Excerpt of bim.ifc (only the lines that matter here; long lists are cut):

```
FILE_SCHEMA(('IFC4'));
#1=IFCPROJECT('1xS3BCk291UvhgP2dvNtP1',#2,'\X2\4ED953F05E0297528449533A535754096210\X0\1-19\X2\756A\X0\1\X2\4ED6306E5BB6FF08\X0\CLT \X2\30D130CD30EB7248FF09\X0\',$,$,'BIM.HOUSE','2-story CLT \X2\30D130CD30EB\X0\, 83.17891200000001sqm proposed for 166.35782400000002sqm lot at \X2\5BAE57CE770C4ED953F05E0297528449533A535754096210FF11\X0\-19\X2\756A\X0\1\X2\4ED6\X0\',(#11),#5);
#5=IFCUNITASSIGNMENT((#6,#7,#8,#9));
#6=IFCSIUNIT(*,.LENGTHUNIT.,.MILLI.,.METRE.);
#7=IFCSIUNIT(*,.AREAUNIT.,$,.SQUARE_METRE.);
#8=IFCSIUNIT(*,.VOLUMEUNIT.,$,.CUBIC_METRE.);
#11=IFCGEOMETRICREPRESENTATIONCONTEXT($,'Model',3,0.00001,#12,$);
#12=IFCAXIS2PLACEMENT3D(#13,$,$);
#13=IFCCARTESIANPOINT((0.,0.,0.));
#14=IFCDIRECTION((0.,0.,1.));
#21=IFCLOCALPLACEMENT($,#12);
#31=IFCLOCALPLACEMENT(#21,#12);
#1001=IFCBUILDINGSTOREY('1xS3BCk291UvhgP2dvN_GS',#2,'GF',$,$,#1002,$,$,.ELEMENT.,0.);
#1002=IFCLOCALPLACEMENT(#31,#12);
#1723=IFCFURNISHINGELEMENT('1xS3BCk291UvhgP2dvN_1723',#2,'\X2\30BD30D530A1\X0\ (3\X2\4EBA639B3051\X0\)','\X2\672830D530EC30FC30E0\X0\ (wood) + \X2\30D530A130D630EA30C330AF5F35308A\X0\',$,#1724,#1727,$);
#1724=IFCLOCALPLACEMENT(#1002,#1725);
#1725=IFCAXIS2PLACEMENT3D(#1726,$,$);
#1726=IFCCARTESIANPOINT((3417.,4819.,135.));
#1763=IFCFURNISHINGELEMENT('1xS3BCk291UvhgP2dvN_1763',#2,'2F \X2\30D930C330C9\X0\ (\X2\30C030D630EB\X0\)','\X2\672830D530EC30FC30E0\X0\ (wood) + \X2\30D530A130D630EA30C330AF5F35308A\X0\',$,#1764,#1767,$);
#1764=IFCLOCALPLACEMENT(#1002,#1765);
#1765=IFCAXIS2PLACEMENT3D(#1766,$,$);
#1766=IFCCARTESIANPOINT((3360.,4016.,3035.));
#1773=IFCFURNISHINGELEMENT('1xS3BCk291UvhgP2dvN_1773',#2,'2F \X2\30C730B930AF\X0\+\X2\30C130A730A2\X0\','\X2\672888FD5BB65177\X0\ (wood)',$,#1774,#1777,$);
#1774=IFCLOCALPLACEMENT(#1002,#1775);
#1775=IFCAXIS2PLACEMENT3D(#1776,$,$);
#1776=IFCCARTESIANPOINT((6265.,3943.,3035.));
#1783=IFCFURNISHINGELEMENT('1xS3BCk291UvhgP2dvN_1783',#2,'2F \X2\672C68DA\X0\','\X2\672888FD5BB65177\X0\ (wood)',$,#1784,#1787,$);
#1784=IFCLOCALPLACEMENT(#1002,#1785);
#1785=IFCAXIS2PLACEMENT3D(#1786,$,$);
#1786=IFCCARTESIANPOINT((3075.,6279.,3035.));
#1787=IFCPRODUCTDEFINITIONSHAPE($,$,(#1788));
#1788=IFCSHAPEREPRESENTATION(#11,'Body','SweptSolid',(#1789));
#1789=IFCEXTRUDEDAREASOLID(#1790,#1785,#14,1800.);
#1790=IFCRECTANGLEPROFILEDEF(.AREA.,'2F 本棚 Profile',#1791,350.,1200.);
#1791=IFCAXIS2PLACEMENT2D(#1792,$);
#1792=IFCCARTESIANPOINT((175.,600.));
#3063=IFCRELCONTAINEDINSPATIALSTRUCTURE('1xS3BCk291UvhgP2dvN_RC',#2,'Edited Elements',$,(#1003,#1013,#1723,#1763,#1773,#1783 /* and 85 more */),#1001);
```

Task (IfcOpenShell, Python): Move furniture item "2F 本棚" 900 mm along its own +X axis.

```python
import ifcopenshell
import ifcopenshell.api.geometry
import ifcopenshell.util.placement
import ifcopenshell.util.unit

model = ifcopenshell.open("bim.ifc")
unit_scale = ifcopenshell.util.unit.calculate_unit_scale(model)

item = model.by_id(1783)
matrix = ifcopenshell.util.placement.get_local_placement(item.ObjectPlacement)
matrix[:3, 3] += matrix[:3, 0] * 0.9 / unit_scale
ifcopenshell.api.geometry.edit_object_placement(model, product=item, matrix=matrix, is_si=False)

print(ifcopenshell.util.placement.get_local_placement(item.ObjectPlacement).round(3) + 0.0)

model.write("bim-out.ifc")
```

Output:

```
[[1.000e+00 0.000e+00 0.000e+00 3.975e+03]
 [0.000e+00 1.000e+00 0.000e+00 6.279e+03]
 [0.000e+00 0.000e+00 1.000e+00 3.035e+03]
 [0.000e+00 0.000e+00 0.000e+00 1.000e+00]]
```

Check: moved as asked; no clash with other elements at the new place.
